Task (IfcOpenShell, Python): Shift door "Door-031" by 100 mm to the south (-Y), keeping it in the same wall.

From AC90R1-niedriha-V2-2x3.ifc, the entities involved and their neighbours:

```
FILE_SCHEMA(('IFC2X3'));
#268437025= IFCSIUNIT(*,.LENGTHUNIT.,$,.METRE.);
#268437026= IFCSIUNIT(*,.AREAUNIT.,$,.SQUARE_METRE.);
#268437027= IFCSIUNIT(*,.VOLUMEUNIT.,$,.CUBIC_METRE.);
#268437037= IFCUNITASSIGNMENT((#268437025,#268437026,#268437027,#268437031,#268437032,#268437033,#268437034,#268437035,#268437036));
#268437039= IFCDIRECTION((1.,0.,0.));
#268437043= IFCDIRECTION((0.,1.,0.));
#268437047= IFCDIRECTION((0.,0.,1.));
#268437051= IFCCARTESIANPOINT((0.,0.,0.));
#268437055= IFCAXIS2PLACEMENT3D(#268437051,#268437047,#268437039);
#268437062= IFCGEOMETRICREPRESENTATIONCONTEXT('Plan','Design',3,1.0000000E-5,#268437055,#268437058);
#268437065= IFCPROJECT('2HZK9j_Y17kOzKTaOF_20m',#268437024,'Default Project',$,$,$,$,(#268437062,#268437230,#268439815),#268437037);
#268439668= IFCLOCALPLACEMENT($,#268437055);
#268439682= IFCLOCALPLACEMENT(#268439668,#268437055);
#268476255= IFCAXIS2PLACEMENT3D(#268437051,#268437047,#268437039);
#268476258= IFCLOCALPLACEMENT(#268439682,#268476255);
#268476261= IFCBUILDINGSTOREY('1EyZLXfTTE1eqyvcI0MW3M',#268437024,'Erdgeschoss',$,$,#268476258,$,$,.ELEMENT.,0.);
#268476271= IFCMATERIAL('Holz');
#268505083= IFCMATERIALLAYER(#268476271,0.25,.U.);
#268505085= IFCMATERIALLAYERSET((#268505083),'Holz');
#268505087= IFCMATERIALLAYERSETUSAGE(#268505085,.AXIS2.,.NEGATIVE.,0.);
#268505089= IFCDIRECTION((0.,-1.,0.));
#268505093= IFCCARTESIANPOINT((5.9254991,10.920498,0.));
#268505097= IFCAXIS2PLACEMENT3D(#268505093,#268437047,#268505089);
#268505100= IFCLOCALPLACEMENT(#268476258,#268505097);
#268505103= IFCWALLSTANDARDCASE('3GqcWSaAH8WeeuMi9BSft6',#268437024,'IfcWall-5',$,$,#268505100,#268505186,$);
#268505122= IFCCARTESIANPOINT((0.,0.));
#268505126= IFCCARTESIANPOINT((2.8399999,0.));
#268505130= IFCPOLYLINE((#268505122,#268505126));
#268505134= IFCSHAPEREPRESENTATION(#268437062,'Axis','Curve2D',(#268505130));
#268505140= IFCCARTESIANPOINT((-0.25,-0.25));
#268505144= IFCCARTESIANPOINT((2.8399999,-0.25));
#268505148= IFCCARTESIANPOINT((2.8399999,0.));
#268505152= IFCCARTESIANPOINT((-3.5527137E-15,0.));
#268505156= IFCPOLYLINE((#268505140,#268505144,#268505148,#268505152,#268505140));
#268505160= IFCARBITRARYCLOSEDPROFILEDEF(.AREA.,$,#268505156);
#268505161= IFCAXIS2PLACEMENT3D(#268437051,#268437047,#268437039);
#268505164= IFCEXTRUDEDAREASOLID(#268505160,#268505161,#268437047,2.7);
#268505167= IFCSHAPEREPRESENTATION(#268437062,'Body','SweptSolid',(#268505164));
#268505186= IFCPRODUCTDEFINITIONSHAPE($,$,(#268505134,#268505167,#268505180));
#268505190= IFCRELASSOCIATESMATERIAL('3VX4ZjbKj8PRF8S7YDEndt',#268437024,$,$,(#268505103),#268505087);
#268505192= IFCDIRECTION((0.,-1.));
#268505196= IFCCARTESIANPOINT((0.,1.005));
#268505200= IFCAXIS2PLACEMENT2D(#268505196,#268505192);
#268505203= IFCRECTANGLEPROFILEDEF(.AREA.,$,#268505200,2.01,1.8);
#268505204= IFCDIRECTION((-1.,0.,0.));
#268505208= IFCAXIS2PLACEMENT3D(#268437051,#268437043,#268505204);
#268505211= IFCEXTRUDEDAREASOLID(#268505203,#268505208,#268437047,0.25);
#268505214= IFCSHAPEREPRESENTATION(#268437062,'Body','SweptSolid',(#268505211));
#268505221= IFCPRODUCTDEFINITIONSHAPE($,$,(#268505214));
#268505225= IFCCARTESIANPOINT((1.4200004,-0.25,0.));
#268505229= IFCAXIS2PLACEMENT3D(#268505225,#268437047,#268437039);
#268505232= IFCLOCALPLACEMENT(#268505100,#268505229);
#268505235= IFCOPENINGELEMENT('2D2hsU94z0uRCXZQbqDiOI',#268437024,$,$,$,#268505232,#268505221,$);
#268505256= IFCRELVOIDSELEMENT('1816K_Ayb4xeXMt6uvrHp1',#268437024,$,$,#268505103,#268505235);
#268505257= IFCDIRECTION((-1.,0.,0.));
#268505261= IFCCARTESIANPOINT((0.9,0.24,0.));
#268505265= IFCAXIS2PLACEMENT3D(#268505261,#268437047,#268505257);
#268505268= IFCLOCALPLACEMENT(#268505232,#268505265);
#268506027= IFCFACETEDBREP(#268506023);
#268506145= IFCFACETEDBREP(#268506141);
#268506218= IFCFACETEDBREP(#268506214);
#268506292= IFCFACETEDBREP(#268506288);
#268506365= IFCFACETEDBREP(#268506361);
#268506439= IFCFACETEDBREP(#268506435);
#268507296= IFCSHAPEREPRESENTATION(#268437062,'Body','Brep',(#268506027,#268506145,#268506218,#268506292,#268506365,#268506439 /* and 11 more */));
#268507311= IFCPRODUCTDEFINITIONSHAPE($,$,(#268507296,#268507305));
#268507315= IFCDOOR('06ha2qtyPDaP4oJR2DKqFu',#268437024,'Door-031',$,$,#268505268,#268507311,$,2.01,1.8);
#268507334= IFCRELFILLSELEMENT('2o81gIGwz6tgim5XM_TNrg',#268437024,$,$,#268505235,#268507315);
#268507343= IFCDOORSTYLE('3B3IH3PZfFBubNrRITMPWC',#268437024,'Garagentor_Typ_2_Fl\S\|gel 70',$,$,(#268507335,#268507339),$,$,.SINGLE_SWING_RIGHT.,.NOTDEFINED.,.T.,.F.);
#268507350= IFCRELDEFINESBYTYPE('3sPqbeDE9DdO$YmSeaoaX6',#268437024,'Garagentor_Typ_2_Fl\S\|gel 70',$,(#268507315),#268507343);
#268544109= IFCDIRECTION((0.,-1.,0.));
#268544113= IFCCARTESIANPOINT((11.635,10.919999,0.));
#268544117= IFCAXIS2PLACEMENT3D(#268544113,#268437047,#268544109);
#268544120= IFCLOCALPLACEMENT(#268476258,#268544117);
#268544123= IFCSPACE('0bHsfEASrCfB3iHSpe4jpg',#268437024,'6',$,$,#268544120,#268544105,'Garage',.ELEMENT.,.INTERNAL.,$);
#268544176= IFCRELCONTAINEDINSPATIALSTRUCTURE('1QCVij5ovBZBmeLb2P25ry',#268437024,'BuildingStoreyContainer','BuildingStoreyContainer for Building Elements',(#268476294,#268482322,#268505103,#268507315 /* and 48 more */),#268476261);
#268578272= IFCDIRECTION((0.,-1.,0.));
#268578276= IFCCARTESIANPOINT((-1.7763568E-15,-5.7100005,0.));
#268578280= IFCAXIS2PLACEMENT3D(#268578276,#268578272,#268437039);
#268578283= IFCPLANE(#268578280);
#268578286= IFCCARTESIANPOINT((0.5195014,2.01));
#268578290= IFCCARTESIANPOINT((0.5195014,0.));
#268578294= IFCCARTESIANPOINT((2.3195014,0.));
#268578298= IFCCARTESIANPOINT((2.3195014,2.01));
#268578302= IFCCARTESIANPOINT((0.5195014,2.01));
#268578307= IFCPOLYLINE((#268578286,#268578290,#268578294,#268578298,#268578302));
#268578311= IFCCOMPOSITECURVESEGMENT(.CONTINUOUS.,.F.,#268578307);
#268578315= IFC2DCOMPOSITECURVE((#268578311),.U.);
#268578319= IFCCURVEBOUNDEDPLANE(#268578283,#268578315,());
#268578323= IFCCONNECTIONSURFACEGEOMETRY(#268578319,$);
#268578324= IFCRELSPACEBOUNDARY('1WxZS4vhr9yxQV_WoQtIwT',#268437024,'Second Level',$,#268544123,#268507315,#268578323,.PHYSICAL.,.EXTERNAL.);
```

```python
import numpy as np
import ifcopenshell
import ifcopenshell.api.geometry
import ifcopenshell.util.placement
import ifcopenshell.util.unit

model = ifcopenshell.open("AC90R1-niedriha-V2-2x3.ifc")
unit_scale = ifcopenshell.util.unit.calculate_unit_scale(model)

door = model.by_guid("06ha2qtyPDaP4oJR2DKqFu")
opening = door.FillsVoids[0].RelatingOpeningElement
wall = opening.VoidsElements[0].RelatingBuildingElement

wall_matrix = ifcopenshell.util.placement.get_local_placement(wall.ObjectPlacement)
shift = wall_matrix[:3, 0] * 0.1 / unit_scale
before = ifcopenshell.util.placement.get_local_placement(door.ObjectPlacement)[:3, 3].copy()

# The door is placed relative to its opening, so it follows when the opening moves.
matrix = ifcopenshell.util.placement.get_local_placement(opening.ObjectPlacement)
matrix[:3, 3] += shift
ifcopenshell.api.geometry.edit_object_placement(
    model, product=opening, matrix=matrix, is_si=False, should_transform_children=True
)

# Space boundary surfaces are stored in each space's coordinates; move them too.
for rel in door.ProvidesBoundaries:
    if not rel.ConnectionGeometry:
        continue
    surface = rel.ConnectionGeometry.SurfaceOnRelatingElement.BasisSurface
    space_matrix = ifcopenshell.util.placement.get_local_placement(rel.RelatingSpace.ObjectPlacement)
    point = np.array(surface.Position.Location.Coordinates) + space_matrix[:3, :3].T @ shift
    surface.Position = model.createIfcAxis2Placement3D(
        model.createIfcCartesianPoint(point.tolist()), surface.Position.Axis, surface.Position.RefDirection
    )

after = ifcopenshell.util.placement.get_local_placement(door.ObjectPlacement)[:3, 3]
print("door moved by", (after - before).round(3) + 0.0)

model.write("AC90R1-niedriha-V2-2x3_v2.ifc")
```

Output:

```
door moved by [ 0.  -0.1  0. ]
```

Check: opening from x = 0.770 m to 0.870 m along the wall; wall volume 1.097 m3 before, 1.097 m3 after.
